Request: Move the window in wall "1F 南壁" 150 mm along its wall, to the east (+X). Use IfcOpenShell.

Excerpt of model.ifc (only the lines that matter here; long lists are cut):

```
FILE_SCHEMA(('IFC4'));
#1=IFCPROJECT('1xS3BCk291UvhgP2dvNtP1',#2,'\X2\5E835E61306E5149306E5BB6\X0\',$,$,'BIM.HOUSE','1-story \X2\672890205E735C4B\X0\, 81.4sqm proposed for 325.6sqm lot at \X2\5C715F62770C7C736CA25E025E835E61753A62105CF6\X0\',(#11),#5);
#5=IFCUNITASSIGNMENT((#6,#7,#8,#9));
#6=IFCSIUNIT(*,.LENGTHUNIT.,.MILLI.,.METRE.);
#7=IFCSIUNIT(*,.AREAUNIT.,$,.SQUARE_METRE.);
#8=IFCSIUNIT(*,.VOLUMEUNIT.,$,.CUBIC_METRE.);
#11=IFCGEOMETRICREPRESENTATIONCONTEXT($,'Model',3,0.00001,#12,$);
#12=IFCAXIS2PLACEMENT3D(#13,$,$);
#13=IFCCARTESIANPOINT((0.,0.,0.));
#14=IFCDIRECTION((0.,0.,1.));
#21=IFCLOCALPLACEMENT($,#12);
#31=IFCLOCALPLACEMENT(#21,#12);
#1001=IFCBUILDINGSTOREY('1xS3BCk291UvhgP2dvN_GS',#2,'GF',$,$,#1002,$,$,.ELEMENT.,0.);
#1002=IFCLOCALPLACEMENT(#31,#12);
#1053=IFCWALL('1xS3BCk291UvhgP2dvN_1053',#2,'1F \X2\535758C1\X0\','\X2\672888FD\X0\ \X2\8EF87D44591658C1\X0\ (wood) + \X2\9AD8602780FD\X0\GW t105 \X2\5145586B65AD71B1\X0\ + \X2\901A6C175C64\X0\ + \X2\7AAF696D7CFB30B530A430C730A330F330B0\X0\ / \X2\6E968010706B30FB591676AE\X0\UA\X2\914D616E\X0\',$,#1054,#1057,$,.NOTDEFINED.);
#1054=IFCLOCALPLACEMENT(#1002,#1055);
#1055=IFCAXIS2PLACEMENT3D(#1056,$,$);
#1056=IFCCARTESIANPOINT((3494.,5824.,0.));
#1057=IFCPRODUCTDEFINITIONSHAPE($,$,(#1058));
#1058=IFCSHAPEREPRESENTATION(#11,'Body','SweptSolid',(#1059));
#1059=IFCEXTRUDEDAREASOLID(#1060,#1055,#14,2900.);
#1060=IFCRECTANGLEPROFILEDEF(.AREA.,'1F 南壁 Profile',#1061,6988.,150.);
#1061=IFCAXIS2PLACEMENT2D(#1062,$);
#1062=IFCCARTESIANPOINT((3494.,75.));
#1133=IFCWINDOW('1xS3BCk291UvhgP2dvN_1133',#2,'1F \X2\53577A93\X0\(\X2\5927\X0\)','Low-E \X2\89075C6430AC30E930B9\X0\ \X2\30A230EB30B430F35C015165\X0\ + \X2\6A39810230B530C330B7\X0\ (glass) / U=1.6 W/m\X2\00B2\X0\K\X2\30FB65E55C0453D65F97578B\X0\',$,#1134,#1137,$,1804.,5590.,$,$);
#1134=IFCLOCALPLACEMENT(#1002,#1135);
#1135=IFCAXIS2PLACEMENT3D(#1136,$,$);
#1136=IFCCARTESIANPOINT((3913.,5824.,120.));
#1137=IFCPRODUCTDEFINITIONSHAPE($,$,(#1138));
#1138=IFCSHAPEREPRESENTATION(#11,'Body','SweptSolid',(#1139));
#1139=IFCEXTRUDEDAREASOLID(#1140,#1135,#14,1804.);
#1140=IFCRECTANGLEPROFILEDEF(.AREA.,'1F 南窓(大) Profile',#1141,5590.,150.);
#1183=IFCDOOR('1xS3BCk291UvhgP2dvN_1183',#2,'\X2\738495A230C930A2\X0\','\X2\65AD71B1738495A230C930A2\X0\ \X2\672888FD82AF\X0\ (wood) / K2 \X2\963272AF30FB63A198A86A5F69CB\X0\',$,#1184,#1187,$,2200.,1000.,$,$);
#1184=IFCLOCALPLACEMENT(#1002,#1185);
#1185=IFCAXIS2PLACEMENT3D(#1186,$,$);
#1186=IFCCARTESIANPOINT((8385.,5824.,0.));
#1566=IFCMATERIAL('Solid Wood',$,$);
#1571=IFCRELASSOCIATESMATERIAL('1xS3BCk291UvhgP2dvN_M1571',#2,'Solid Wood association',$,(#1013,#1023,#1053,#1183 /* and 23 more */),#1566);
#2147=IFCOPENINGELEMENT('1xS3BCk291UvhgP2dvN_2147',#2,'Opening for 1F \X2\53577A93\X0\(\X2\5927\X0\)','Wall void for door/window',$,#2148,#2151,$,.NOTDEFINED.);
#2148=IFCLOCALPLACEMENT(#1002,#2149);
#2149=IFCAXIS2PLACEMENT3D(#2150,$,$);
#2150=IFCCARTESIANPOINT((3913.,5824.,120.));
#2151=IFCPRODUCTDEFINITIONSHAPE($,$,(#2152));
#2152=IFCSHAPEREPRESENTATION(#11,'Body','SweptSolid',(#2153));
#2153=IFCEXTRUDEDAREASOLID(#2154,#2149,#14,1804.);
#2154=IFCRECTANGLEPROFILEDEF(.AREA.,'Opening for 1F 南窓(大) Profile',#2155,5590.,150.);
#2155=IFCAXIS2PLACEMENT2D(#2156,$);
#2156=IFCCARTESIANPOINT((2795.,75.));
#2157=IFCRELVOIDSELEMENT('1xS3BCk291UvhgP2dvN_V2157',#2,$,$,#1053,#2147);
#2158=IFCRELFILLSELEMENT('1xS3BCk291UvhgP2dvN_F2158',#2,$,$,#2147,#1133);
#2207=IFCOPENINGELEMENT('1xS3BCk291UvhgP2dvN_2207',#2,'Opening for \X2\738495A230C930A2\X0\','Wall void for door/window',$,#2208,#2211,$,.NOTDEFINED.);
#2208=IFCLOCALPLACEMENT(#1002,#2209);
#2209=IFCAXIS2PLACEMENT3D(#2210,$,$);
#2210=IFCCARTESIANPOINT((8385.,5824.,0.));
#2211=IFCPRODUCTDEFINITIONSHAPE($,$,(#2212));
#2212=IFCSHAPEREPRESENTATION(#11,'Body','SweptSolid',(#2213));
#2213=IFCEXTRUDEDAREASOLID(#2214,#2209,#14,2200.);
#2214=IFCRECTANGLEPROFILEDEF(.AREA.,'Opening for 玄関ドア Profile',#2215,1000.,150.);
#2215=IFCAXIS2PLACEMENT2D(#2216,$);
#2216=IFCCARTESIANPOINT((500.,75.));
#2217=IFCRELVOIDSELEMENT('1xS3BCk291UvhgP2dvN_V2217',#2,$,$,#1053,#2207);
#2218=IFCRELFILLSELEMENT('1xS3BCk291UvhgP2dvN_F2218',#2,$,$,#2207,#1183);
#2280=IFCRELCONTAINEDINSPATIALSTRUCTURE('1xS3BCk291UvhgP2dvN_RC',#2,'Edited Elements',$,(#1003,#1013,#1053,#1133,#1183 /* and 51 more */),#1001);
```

```python
import ifcopenshell
import ifcopenshell.api.geometry
import ifcopenshell.util.placement
import ifcopenshell.util.unit

model = ifcopenshell.open("model.ifc")
unit_scale = ifcopenshell.util.unit.calculate_unit_scale(model)

window = model.by_id(1133)
opening = window.FillsVoids[0].RelatingOpeningElement
wall = opening.VoidsElements[0].RelatingBuildingElement

wall_matrix = ifcopenshell.util.placement.get_local_placement(wall.ObjectPlacement)
shift = wall_matrix[:3, 0] * 0.15 / unit_scale
before = ifcopenshell.util.placement.get_local_placement(window.ObjectPlacement)[:3, 3].copy()

# The window is not placed relative to its opening, so move both.
for product in (opening, window):
    matrix = ifcopenshell.util.placement.get_local_placement(product.ObjectPlacement)
    matrix[:3, 3] += shift
    ifcopenshell.api.geometry.edit_object_placement(model, product=product, matrix=matrix, is_si=False)

after = ifcopenshell.util.placement.get_local_placement(window.ObjectPlacement)[:3, 3]
print("window moved by", (after - before).round(3) + 0.0)

model.write("model-out.ifc")
```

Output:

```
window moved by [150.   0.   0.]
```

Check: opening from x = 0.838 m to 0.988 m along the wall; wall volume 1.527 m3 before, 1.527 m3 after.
